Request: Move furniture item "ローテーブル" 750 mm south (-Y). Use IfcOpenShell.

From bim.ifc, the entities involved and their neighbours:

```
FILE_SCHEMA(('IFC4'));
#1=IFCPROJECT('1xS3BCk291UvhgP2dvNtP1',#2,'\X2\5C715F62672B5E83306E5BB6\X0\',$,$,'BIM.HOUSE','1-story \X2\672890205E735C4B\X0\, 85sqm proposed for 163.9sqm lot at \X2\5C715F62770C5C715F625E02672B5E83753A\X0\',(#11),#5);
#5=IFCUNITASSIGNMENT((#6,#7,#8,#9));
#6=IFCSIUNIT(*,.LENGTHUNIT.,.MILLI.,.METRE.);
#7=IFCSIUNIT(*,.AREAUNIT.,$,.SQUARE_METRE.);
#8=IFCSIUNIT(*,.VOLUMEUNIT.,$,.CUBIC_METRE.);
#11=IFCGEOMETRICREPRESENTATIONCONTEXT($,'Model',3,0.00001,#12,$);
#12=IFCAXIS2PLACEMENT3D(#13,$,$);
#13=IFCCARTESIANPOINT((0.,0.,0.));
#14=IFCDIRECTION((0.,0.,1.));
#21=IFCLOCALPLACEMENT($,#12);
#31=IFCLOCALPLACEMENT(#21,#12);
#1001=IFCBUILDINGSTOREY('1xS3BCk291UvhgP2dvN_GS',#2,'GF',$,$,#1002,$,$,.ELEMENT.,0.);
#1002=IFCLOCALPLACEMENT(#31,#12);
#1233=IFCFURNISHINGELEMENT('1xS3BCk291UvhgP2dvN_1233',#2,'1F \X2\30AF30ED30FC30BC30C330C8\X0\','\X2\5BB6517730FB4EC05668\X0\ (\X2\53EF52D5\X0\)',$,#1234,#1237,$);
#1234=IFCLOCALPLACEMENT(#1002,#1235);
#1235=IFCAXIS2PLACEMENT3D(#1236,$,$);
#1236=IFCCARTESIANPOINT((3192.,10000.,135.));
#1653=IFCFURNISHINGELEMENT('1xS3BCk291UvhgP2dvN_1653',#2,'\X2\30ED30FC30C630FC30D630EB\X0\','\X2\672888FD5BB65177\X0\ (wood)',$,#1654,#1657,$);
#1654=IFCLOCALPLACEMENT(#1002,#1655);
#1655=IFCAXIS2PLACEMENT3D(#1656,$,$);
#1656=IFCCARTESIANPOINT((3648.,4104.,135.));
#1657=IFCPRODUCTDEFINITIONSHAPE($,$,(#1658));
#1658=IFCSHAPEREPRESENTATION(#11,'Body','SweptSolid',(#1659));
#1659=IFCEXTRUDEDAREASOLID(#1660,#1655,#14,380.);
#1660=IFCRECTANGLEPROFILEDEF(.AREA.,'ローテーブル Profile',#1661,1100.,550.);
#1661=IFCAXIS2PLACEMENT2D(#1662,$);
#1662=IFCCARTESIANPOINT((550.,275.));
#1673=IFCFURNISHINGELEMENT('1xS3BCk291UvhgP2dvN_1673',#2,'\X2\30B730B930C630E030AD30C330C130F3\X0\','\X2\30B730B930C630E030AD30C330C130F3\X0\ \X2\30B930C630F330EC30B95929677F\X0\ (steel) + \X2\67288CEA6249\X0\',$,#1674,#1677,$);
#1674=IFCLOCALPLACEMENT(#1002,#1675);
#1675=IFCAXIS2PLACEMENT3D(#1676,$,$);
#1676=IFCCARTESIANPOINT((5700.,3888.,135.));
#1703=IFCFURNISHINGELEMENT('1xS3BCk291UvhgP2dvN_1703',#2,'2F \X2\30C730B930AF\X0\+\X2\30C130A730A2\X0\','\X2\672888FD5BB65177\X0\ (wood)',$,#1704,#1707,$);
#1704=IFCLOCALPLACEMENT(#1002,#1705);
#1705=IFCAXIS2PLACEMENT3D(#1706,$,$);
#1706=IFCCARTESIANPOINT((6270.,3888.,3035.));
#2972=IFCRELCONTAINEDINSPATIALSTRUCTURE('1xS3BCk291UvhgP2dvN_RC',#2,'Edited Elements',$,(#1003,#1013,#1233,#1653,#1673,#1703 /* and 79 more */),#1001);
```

```python
import ifcopenshell
import ifcopenshell.api.geometry
import ifcopenshell.util.placement
import ifcopenshell.util.unit

model = ifcopenshell.open("bim.ifc")
unit_scale = ifcopenshell.util.unit.calculate_unit_scale(model)

item = model.by_id(1653)
matrix = ifcopenshell.util.placement.get_local_placement(item.ObjectPlacement)
matrix[1, 3] -= 0.75 / unit_scale
ifcopenshell.api.geometry.edit_object_placement(model, product=item, matrix=matrix, is_si=False)

print(ifcopenshell.util.placement.get_local_placement(item.ObjectPlacement).round(3) + 0.0)

model.write("bim-out.ifc")
```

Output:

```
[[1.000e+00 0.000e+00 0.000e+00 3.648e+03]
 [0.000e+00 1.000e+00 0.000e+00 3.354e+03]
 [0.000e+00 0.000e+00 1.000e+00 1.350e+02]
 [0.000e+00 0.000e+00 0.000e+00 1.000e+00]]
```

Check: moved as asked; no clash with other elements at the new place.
